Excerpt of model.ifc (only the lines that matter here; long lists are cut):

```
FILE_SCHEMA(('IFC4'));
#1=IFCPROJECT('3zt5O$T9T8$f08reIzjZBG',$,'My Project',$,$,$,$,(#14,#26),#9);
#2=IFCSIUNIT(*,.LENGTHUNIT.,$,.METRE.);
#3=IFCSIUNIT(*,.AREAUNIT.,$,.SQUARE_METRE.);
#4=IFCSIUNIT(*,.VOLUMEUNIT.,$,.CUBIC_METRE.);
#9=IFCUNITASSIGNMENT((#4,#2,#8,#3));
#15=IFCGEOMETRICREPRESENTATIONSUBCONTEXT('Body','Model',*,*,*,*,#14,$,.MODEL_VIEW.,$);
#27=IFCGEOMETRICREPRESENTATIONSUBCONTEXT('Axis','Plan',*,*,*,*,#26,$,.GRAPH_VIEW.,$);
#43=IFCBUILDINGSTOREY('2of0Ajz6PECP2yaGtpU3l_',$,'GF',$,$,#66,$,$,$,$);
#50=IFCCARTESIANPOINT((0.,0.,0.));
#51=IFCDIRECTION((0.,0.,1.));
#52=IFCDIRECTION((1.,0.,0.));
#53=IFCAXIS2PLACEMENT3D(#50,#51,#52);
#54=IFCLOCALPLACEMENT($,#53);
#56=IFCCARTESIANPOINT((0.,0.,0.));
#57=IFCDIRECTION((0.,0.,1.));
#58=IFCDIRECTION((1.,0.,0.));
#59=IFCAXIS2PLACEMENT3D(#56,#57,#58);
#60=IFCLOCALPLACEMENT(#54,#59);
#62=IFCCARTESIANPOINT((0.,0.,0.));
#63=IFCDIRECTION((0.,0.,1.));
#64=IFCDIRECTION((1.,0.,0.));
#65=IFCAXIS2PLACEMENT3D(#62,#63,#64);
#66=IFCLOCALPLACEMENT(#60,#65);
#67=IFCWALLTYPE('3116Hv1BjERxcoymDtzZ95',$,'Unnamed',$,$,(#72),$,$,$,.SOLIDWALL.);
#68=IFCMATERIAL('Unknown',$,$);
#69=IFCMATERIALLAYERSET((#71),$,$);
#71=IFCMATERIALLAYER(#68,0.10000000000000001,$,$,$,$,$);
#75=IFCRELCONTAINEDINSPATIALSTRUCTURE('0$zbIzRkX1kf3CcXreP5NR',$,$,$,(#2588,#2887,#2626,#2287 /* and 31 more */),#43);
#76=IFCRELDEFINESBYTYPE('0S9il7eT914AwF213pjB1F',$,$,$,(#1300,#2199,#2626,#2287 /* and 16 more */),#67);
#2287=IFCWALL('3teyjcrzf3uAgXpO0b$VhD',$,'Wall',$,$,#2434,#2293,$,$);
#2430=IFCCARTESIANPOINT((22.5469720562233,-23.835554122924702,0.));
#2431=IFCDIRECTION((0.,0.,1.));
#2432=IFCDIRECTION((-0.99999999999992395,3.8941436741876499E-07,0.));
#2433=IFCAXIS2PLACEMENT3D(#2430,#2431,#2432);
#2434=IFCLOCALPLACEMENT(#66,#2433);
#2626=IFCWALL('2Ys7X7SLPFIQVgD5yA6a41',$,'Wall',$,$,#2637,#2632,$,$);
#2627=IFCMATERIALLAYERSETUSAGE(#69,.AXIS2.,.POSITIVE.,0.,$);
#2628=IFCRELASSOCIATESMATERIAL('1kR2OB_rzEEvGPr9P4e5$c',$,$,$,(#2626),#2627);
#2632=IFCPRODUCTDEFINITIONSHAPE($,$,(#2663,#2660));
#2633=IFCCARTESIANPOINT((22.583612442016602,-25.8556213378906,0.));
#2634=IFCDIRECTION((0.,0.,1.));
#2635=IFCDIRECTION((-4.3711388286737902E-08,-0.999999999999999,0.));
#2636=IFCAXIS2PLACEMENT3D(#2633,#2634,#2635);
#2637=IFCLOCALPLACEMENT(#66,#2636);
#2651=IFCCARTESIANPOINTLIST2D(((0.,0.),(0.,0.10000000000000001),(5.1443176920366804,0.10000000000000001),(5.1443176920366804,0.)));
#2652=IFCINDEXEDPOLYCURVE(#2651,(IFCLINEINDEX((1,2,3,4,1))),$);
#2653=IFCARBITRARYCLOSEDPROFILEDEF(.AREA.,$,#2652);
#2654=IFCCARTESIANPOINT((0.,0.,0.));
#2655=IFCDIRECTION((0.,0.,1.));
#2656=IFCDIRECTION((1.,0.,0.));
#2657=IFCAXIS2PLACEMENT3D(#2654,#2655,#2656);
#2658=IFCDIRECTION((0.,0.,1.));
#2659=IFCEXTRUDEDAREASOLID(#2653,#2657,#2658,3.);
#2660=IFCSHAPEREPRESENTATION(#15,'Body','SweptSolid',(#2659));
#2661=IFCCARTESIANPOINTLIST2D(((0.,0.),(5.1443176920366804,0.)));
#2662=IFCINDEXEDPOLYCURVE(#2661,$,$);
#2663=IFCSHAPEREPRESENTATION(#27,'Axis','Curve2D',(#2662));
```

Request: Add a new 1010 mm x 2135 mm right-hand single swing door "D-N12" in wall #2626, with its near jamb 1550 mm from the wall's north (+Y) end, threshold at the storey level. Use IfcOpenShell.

```python
import numpy as np
import ifcopenshell
import ifcopenshell.api.feature
import ifcopenshell.api.geometry
import ifcopenshell.api.root
import ifcopenshell.api.spatial
import ifcopenshell.geom
import ifcopenshell.util.element
import ifcopenshell.util.placement
import ifcopenshell.util.representation
import ifcopenshell.util.shape
import ifcopenshell.util.unit

model = ifcopenshell.open("model.ifc")
unit_scale = ifcopenshell.util.unit.calculate_unit_scale(model)
settings = ifcopenshell.geom.settings()


def volume(element):
    """Net volume in cubic metres, openings subtracted."""
    shape = ifcopenshell.geom.create_shape(settings, element)
    return ifcopenshell.util.shape.get_volume(shape.geometry)


wall = model.by_guid("2Ys7X7SLPFIQVgD5yA6a41")
storey = ifcopenshell.util.element.get_container(wall, ifc_class="IfcBuildingStorey")
context = ifcopenshell.util.representation.get_context(model, "Model", "Body", "MODEL_VIEW")
before = volume(wall)

width, height, from_end, sill = 1.01, 2.135, 1.55, 0.0  # metres

# The wall runs along its own X axis, and the end named is its -X end.
wall_shape = ifcopenshell.geom.create_shape(settings, wall)
x, y, z = ifcopenshell.util.shape.get_vertices(wall_shape.geometry).T
start = x.min() + from_end
face, thickness = float(y.min()), float(y.max() - y.min())
wall_matrix = ifcopenshell.util.placement.get_local_placement(wall.ObjectPlacement)
level = ifcopenshell.util.placement.get_local_placement(storey.ObjectPlacement)[2, 3]


def in_wall(x, y):
    """Placement at x, y metres in the wall's axes, at sill height."""
    matrix = wall_matrix.copy()
    matrix[:, 3] = wall_matrix @ np.array([x / unit_scale, y / unit_scale, 0.0, 1.0])
    matrix[2, 3] = level + sill / unit_scale
    return matrix


# Opening: a box that overshoots both wall faces by 50 mm.
opening = ifcopenshell.api.root.create_entity(model, ifc_class="IfcOpeningElement", predefined_type="OPENING")
box = ifcopenshell.api.geometry.add_wall_representation(
    model, context=context, length=width, height=height, thickness=thickness + 0.1
)
ifcopenshell.api.geometry.assign_representation(model, product=opening, representation=box)
ifcopenshell.api.geometry.edit_object_placement(model, product=opening, matrix=in_wall(start, face - 0.05), is_si=False)
ifcopenshell.api.feature.add_feature(model, feature=opening, element=wall)

door = ifcopenshell.api.root.create_entity(model, ifc_class="IfcDoor", name="D-N12", predefined_type="DOOR")
door.OverallWidth, door.OverallHeight = width / unit_scale, height / unit_scale
door.OperationType = "SINGLE_SWING_RIGHT"
body = ifcopenshell.api.geometry.add_door_representation(
    model,
    context=context,
    overall_width=door.OverallWidth,
    overall_height=door.OverallHeight,
    operation_type="SINGLE_SWING_RIGHT",
    lining_properties={"LiningDepth": thickness / unit_scale, "ThresholdDepth": thickness / unit_scale},
)
ifcopenshell.api.geometry.assign_representation(model, product=door, representation=body)
ifcopenshell.api.spatial.assign_container(model, products=[door], relating_structure=storey)
ifcopenshell.api.feature.add_filling(model, opening=opening, element=door)

# The lining spans the wall, so the door starts at the wall face.
ifcopenshell.api.geometry.edit_object_placement(model, product=door, matrix=in_wall(start, face), is_si=False)

after = volume(wall)

print(f"wall volume {before:.3f} -> {after:.3f} m3")

model.write("model_edited.ifc")
```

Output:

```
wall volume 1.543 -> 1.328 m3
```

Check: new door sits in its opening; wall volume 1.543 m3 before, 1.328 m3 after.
